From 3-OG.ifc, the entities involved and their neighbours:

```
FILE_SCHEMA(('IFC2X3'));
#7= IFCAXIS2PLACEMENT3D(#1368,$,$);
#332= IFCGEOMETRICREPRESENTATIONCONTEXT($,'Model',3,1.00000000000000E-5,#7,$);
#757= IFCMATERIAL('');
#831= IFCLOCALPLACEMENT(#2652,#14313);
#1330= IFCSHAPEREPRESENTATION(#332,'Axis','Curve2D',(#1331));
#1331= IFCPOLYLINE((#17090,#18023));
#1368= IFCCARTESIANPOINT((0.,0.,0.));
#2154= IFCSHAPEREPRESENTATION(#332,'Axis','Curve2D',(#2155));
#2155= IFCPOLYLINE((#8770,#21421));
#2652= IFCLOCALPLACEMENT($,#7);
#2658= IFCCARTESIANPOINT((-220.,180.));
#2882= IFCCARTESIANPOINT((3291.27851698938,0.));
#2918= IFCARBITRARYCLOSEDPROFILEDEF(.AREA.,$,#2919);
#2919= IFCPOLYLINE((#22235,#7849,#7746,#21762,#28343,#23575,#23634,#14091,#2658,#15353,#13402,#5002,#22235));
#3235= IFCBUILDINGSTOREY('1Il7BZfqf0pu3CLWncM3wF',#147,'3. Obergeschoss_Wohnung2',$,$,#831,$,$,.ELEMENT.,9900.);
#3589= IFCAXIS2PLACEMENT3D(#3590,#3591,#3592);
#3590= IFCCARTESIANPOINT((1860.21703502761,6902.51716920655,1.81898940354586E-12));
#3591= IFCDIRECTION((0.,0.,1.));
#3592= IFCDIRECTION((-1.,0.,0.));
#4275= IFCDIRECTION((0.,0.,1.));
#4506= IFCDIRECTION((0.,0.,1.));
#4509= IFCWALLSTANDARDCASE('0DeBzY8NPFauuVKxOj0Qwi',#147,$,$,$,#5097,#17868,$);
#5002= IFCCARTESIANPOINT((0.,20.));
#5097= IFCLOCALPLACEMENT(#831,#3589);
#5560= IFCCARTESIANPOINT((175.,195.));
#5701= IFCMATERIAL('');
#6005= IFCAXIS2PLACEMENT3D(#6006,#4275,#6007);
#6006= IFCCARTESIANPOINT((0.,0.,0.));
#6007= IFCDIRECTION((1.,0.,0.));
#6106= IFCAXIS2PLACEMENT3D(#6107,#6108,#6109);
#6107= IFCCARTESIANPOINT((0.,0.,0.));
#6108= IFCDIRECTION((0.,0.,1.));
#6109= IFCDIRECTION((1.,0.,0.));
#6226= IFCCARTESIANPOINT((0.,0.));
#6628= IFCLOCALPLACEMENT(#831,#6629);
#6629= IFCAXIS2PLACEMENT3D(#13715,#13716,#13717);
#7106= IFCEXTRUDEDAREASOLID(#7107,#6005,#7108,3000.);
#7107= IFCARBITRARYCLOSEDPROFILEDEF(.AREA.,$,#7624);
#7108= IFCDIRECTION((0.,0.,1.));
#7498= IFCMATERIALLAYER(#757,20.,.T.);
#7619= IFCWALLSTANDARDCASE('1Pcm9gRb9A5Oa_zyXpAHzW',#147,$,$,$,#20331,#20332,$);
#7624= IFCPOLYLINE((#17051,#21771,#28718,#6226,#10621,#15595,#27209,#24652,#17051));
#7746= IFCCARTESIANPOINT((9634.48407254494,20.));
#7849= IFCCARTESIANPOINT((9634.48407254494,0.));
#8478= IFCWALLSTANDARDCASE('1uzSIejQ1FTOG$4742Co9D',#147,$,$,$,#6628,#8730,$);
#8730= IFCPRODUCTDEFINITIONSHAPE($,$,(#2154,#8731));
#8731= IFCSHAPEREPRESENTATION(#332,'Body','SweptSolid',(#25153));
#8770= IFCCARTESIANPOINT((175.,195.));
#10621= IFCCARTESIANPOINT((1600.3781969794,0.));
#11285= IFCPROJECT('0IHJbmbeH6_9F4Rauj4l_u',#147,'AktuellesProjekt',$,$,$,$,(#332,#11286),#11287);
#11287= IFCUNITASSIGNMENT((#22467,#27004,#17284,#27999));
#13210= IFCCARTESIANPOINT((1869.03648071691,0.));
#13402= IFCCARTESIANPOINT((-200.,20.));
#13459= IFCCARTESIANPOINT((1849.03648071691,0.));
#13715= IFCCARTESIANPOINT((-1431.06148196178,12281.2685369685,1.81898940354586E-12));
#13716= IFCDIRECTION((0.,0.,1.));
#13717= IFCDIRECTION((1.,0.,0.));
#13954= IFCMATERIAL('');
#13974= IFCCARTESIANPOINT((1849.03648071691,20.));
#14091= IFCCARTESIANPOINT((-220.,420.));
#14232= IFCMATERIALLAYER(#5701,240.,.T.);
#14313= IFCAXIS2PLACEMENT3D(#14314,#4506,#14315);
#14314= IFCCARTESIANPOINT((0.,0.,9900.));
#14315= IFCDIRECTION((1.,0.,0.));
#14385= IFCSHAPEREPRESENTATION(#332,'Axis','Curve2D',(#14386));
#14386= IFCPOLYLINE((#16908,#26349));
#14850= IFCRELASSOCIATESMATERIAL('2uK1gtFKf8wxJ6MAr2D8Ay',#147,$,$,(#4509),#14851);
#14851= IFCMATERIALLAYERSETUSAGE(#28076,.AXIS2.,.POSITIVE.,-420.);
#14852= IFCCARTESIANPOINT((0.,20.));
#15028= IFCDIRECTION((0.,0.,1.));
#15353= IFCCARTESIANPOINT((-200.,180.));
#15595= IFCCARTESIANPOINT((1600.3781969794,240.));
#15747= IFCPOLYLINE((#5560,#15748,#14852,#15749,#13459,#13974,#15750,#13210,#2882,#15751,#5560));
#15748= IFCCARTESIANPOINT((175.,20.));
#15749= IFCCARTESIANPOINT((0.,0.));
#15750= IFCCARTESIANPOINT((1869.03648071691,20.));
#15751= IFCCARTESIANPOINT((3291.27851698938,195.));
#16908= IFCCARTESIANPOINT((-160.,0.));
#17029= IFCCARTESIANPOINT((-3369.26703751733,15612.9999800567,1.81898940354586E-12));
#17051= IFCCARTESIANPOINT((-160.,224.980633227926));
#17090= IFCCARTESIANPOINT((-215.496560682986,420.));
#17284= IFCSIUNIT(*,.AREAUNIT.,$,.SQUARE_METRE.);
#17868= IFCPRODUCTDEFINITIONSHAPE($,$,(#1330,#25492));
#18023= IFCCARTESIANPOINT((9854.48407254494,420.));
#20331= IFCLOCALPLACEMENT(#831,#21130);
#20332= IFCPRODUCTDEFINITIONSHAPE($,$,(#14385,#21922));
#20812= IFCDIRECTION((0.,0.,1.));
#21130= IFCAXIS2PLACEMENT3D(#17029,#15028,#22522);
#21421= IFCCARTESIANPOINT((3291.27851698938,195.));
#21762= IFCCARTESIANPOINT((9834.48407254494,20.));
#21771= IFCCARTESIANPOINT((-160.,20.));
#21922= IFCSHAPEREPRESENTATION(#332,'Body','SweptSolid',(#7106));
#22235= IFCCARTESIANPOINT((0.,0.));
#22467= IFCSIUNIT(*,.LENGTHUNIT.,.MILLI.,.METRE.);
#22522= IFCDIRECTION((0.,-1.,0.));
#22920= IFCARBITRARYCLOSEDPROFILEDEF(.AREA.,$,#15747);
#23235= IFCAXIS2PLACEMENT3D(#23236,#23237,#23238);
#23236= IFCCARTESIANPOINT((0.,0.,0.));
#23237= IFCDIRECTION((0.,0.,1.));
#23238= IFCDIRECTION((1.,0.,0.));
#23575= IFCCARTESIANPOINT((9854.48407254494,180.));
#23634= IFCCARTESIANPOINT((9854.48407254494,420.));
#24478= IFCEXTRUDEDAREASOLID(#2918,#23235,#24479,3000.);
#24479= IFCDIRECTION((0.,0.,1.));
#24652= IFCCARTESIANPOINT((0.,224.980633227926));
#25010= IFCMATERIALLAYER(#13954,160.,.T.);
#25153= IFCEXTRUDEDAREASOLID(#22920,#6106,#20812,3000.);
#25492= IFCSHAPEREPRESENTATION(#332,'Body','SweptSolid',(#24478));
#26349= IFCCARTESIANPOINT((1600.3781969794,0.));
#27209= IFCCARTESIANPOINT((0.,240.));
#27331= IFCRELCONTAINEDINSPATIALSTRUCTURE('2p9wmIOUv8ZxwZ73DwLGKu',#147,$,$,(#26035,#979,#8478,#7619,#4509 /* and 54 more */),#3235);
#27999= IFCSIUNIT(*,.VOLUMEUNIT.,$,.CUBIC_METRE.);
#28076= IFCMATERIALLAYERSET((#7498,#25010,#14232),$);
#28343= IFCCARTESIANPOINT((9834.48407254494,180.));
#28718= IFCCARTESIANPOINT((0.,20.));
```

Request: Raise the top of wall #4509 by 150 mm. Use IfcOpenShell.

```python
import ifcopenshell
import ifcopenshell.geom
import ifcopenshell.util.shape

model = ifcopenshell.open("3-OG.ifc")
settings = ifcopenshell.geom.settings()


def volume(element):
    """Net volume in cubic metres, openings subtracted."""
    shape = ifcopenshell.geom.create_shape(settings, element)
    return ifcopenshell.util.shape.get_volume(shape.geometry)


wall = model.by_guid("0DeBzY8NPFauuVKxOj0Qwi")
before = volume(wall)

body = next(r for r in wall.Representation.Representations if r.RepresentationIdentifier == "Body")
solid = body.Items[0]
old_height = solid.Depth
solid.Depth += 150.0
after = volume(wall)

print(f"height {old_height:g} -> {solid.Depth:g}, volume {before:.3f} -> {after:.3f} m3")

model.write("3-OG_rev.ifc")
```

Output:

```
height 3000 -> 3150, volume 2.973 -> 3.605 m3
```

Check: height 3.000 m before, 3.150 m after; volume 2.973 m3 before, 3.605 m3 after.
